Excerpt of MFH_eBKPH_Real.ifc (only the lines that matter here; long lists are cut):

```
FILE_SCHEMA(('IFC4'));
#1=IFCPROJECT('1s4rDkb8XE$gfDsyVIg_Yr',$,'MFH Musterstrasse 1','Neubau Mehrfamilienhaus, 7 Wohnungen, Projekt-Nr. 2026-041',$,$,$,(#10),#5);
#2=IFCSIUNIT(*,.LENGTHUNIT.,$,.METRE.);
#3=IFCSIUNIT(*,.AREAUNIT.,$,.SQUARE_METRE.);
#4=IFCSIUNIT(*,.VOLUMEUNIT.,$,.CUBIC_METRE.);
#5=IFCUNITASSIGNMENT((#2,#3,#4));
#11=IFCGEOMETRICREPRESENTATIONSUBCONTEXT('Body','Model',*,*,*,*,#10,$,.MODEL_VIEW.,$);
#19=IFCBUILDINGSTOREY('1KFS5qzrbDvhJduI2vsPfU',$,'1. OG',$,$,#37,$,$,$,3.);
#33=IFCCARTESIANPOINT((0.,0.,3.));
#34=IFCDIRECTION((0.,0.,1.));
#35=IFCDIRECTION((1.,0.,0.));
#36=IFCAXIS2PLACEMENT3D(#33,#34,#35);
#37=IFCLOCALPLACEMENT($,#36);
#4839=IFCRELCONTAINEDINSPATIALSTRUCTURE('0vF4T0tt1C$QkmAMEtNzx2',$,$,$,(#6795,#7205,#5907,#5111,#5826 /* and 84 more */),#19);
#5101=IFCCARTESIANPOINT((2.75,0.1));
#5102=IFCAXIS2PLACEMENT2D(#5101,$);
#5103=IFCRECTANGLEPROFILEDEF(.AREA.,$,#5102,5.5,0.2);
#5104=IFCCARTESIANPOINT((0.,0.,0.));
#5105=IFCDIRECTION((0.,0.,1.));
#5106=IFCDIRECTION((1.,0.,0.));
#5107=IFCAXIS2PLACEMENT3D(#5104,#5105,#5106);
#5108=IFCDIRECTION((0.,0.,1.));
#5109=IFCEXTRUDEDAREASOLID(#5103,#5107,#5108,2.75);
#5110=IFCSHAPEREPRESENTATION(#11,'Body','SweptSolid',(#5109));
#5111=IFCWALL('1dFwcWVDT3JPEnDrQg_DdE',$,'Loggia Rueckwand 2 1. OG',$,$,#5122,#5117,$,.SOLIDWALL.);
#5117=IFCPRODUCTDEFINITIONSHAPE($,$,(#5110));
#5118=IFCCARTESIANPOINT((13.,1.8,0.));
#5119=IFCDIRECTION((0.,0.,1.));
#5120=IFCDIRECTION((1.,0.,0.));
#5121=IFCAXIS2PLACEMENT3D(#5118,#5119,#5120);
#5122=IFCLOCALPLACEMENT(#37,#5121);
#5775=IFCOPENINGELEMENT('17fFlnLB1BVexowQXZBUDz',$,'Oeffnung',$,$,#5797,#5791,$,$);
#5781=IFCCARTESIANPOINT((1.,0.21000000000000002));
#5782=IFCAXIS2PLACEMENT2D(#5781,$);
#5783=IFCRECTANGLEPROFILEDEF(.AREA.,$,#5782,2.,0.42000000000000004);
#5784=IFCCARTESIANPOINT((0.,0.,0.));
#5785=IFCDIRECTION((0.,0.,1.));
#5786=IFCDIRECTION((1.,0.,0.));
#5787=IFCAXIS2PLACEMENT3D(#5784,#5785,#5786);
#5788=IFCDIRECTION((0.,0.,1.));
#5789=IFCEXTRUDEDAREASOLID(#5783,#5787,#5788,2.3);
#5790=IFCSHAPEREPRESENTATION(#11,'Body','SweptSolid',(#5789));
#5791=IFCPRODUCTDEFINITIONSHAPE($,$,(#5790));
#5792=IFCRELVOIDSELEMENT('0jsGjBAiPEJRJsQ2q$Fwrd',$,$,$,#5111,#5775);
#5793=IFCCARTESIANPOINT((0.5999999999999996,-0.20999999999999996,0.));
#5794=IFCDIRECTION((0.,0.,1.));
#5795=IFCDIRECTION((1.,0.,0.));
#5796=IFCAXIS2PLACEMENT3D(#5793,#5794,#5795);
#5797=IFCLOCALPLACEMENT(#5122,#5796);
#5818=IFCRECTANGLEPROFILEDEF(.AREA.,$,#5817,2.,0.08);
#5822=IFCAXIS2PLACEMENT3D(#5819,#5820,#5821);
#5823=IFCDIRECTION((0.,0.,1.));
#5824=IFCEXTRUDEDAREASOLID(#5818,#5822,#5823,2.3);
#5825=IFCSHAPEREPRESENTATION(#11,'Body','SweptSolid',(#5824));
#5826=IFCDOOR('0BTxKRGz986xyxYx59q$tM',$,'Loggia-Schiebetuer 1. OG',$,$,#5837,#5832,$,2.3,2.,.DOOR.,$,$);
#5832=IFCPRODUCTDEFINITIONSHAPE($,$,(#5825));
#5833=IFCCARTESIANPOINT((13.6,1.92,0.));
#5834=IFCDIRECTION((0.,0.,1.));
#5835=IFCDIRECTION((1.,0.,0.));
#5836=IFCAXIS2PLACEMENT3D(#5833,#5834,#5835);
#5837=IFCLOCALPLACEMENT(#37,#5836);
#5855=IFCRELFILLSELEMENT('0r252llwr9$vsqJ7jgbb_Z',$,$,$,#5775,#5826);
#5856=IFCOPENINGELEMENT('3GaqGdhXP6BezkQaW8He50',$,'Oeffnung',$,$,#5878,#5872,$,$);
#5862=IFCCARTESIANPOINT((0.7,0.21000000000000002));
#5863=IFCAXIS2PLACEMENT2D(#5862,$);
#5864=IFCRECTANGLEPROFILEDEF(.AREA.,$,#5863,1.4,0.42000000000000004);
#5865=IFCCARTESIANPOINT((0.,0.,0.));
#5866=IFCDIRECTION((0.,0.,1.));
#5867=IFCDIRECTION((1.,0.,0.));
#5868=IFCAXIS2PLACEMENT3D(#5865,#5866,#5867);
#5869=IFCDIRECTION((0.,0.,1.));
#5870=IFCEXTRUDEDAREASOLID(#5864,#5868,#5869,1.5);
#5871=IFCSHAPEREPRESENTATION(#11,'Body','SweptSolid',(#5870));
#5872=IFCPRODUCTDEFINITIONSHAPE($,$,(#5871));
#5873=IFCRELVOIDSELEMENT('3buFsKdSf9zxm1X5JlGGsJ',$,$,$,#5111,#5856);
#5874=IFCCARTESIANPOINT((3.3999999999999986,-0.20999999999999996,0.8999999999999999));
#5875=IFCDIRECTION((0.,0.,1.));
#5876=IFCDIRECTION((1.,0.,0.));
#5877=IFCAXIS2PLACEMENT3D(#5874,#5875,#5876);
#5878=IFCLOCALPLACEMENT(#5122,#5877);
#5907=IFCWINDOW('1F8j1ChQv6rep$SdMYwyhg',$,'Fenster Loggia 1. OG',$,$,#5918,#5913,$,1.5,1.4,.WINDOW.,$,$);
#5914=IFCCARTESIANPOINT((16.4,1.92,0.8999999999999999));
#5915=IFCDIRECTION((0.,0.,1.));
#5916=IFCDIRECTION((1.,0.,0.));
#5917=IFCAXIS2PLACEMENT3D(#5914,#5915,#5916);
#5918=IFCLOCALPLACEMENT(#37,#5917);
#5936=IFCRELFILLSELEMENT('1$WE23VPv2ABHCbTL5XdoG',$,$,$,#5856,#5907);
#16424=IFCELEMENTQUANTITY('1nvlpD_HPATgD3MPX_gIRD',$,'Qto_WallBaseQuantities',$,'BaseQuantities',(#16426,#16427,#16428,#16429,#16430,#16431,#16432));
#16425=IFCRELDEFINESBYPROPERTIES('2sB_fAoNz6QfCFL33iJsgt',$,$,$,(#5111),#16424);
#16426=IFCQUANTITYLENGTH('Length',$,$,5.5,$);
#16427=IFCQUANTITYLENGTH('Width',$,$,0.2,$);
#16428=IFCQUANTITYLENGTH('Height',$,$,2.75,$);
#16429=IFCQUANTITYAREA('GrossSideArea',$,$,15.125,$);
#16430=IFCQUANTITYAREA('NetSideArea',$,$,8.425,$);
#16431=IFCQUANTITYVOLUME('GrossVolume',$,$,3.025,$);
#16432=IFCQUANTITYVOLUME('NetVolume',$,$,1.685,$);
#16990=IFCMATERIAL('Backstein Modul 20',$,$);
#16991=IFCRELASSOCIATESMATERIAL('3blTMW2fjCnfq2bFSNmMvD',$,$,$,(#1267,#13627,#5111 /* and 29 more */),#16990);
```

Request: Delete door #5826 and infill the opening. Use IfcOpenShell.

```python
import ifcopenshell
import ifcopenshell.api.feature
import ifcopenshell.api.pset
import ifcopenshell.api.root
import ifcopenshell.geom
import ifcopenshell.util.element
import ifcopenshell.util.shape
import ifcopenshell.util.unit

model = ifcopenshell.open("MFH_eBKPH_Real.ifc")
area_scale = ifcopenshell.util.unit.calculate_unit_scale(model, "AREAUNIT")
volume_scale = ifcopenshell.util.unit.calculate_unit_scale(model, "VOLUMEUNIT")
settings = ifcopenshell.geom.settings()


def volume(element):
    """Net volume in cubic metres, openings subtracted."""
    shape = ifcopenshell.geom.create_shape(settings, element)
    return ifcopenshell.util.shape.get_volume(shape.geometry)


door = model.by_guid("0BTxKRGz986xyxYx59q$tM")
opening = door.FillsVoids[0].RelatingOpeningElement
wall = opening.VoidsElements[0].RelatingBuildingElement
before = volume(wall)

ifcopenshell.api.root.remove_product(model, product=door)
ifcopenshell.api.feature.remove_feature(model, feature=opening)

after = volume(wall)
thickness = 0.2  # wall thickness in metres

# Update the wall's stored quantities.
qto = model.by_id(ifcopenshell.util.element.get_pset(wall, "Qto_WallBaseQuantities", should_inherit=False)["id"])
ifcopenshell.api.pset.edit_qto(model, qto=qto, properties={
    "NetSideArea": after / thickness / area_scale,
    "NetVolume": after / volume_scale,
})

print(f"wall volume {before:.3f} -> {after:.3f} m3")

model.write("MFH_eBKPH_Real_updated.ifc")
```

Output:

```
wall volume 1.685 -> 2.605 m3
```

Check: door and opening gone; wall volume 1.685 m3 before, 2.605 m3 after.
